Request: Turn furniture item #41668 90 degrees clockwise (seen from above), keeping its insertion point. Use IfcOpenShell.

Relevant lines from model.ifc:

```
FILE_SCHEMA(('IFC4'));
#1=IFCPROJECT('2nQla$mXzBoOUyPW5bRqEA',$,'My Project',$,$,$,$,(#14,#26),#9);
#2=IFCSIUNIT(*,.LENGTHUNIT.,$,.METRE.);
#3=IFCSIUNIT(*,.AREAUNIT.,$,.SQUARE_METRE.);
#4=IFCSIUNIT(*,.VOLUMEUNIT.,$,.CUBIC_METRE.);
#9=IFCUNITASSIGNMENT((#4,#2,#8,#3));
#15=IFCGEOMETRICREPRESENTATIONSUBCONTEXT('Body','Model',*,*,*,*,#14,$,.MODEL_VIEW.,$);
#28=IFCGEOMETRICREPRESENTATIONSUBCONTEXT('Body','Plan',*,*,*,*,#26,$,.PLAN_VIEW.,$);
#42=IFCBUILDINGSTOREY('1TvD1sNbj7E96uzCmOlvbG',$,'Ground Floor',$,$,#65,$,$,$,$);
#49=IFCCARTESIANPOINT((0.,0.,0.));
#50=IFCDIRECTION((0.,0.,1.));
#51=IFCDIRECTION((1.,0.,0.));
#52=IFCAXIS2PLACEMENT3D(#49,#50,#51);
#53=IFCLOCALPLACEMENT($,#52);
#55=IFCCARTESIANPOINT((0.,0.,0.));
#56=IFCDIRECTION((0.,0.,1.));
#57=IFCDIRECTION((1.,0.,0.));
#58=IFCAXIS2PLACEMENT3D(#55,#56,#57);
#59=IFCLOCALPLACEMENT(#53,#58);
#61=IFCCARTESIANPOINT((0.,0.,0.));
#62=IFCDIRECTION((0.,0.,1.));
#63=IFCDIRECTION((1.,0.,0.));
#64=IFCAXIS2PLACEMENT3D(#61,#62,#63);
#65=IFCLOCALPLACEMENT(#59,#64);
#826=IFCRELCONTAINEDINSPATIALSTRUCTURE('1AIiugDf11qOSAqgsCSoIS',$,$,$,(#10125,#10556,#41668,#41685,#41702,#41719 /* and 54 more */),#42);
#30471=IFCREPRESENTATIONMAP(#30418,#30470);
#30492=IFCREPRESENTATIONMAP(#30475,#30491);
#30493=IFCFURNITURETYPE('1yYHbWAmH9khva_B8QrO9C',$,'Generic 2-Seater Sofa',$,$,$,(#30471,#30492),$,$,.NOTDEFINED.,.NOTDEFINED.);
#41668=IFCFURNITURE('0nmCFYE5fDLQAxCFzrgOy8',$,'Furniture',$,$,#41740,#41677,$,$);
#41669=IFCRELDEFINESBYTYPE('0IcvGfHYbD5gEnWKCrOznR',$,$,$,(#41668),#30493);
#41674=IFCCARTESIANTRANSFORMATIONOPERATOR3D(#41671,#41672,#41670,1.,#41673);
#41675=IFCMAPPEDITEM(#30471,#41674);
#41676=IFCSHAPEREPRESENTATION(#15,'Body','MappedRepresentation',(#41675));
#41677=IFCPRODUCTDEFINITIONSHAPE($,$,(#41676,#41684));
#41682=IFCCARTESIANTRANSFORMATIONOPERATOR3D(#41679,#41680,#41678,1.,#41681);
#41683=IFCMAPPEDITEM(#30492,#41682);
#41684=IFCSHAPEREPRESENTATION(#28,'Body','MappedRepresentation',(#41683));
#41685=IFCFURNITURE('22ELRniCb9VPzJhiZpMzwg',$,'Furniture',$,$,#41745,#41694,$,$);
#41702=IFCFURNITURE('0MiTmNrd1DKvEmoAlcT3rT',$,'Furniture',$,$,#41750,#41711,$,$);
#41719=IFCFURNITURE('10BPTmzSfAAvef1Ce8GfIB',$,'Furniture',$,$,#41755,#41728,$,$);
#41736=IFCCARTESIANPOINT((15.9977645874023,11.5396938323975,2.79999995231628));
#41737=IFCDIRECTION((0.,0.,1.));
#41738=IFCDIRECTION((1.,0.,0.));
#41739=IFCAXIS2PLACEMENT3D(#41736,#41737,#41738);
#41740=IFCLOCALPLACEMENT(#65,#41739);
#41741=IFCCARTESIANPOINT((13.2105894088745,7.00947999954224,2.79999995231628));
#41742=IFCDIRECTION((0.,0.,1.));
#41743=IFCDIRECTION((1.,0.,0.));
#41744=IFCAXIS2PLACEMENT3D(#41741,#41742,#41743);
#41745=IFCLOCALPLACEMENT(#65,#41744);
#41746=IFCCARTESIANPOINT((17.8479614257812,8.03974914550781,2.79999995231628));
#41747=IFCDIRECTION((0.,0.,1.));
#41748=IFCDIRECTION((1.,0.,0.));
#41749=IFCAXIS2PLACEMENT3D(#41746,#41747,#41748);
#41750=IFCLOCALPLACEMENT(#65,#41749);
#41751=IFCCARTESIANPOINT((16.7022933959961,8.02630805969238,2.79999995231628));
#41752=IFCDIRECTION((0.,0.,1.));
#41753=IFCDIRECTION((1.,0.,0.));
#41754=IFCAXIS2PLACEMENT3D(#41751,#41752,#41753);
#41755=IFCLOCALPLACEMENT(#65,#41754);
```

```python
import ifcopenshell
import ifcopenshell.api.geometry
import ifcopenshell.util.placement

model = ifcopenshell.open("model.ifc")

item = model.by_guid("0nmCFYE5fDLQAxCFzrgOy8")
matrix = ifcopenshell.util.placement.get_local_placement(item.ObjectPlacement)
matrix = matrix @ ifcopenshell.util.placement.rotation(-90, "Z")
ifcopenshell.api.geometry.edit_object_placement(model, product=item, matrix=matrix, is_si=False)

print(ifcopenshell.util.placement.get_local_placement(item.ObjectPlacement).round(3) + 0.0)

model.write("model_v2.ifc")
```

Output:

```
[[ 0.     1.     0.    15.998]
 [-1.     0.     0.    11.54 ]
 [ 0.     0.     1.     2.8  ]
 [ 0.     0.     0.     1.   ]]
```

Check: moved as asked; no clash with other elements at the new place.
